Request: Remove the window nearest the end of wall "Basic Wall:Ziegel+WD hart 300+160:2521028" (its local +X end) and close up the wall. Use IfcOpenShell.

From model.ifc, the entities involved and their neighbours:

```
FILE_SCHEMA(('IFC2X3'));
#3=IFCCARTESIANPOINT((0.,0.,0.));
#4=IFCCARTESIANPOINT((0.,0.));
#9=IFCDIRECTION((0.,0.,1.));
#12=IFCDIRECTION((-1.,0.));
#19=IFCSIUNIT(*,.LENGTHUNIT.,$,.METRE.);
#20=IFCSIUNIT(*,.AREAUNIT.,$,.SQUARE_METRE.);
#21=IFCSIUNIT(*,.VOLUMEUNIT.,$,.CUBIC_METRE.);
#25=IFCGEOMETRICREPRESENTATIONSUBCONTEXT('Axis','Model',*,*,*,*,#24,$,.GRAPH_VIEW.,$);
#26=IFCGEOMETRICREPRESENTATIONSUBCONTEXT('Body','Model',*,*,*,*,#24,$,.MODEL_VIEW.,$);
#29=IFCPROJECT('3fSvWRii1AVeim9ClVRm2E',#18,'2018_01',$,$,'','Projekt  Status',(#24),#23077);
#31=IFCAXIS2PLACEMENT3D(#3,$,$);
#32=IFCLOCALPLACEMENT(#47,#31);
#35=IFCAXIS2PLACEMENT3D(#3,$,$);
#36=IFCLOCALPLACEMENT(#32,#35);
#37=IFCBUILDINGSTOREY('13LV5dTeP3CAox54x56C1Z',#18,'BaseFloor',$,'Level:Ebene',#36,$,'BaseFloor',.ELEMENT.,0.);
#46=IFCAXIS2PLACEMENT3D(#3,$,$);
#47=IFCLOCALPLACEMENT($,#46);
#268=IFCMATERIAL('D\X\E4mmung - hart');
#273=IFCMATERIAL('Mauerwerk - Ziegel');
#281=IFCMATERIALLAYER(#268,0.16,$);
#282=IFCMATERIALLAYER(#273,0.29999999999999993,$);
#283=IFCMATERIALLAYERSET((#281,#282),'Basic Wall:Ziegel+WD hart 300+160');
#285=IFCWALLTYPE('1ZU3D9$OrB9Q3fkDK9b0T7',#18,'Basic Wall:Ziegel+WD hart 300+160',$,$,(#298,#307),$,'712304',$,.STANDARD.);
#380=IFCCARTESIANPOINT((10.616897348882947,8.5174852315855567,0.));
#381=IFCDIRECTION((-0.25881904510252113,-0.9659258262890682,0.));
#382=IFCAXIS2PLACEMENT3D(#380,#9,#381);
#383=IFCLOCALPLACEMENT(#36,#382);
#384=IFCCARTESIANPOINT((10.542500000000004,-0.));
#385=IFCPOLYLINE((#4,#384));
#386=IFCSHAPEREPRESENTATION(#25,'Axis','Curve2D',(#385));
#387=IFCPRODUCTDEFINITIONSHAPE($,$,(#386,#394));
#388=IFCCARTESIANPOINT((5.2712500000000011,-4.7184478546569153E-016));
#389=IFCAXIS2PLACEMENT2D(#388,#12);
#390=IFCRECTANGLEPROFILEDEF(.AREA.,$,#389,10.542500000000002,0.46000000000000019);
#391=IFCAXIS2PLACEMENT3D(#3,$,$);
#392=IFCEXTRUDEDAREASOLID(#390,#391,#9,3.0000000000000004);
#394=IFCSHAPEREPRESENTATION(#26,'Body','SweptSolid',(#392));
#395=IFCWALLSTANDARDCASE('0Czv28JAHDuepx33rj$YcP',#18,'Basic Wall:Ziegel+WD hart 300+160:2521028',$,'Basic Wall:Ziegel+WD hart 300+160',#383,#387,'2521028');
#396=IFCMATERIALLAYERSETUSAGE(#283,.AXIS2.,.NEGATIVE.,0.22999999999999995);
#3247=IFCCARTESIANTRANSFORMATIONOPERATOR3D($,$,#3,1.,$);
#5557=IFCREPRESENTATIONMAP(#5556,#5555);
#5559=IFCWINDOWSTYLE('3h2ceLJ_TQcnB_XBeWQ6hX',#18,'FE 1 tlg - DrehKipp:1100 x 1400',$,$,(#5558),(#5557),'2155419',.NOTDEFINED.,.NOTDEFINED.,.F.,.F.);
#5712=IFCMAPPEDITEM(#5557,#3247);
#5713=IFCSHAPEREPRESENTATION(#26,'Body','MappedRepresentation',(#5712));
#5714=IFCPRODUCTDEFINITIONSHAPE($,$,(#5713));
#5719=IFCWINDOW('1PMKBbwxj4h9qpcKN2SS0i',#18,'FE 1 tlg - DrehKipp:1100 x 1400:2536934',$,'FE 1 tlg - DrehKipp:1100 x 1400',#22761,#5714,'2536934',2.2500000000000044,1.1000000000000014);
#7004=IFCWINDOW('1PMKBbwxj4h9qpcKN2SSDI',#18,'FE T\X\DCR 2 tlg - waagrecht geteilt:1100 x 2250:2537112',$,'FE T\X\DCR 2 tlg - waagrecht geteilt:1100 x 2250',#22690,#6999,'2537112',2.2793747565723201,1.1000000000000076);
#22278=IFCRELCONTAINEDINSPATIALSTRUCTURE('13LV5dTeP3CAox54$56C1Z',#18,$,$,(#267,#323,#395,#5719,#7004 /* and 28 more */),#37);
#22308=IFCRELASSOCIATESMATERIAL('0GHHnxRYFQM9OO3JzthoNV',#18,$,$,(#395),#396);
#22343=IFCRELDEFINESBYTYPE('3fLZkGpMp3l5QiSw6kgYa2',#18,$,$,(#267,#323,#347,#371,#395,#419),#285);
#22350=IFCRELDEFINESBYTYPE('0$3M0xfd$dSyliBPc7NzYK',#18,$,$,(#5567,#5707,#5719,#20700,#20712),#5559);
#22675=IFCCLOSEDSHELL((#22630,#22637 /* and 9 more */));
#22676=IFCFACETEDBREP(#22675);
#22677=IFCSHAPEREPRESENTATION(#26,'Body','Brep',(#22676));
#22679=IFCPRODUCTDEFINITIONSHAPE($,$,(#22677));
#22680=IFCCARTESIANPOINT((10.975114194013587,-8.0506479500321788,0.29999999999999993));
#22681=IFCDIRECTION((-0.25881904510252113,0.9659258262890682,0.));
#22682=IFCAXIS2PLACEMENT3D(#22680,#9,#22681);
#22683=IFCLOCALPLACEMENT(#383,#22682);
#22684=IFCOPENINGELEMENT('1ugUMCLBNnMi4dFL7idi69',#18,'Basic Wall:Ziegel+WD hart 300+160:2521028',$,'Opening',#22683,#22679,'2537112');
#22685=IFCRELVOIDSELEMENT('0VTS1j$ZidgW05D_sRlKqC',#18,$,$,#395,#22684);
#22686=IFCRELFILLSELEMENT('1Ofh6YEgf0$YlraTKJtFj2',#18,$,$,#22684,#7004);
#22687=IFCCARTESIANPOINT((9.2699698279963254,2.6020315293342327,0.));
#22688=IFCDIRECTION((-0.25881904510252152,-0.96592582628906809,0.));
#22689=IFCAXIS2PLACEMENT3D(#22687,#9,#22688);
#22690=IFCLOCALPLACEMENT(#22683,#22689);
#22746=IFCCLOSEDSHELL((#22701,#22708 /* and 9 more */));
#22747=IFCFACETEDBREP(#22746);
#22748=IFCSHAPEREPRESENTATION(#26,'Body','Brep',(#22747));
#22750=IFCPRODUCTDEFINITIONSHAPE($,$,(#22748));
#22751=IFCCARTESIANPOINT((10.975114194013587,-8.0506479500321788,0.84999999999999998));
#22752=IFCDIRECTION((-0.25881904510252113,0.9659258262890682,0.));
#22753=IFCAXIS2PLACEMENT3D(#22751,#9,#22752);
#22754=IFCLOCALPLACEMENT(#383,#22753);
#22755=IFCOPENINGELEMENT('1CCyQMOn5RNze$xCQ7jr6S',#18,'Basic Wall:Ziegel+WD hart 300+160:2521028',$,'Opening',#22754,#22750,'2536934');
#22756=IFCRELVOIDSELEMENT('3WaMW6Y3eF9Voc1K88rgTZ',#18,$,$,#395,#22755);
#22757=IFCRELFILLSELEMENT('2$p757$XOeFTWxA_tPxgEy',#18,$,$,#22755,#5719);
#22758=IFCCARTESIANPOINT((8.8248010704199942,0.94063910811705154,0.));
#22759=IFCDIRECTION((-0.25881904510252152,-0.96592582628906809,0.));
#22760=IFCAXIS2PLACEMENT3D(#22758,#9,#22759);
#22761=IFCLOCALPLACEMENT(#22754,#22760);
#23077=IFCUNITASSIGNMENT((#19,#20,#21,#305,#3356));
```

```python
import ifcopenshell
import ifcopenshell.api.feature
import ifcopenshell.api.root
import ifcopenshell.geom
import ifcopenshell.util.shape

model = ifcopenshell.open("model.ifc")
settings = ifcopenshell.geom.settings()


def volume(element):
    """Net volume in cubic metres, openings subtracted."""
    shape = ifcopenshell.geom.create_shape(settings, element)
    return ifcopenshell.util.shape.get_volume(shape.geometry)


window = model.by_guid("1PMKBbwxj4h9qpcKN2SS0i")
opening = window.FillsVoids[0].RelatingOpeningElement
wall = opening.VoidsElements[0].RelatingBuildingElement
before = volume(wall)

ifcopenshell.api.root.remove_product(model, product=window)
ifcopenshell.api.feature.remove_feature(model, feature=opening)

after = volume(wall)

print(f"wall volume {before:.3f} -> {after:.3f} m3")

model.write("model_rev.ifc")
```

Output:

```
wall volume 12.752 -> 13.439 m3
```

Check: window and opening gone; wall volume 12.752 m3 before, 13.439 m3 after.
